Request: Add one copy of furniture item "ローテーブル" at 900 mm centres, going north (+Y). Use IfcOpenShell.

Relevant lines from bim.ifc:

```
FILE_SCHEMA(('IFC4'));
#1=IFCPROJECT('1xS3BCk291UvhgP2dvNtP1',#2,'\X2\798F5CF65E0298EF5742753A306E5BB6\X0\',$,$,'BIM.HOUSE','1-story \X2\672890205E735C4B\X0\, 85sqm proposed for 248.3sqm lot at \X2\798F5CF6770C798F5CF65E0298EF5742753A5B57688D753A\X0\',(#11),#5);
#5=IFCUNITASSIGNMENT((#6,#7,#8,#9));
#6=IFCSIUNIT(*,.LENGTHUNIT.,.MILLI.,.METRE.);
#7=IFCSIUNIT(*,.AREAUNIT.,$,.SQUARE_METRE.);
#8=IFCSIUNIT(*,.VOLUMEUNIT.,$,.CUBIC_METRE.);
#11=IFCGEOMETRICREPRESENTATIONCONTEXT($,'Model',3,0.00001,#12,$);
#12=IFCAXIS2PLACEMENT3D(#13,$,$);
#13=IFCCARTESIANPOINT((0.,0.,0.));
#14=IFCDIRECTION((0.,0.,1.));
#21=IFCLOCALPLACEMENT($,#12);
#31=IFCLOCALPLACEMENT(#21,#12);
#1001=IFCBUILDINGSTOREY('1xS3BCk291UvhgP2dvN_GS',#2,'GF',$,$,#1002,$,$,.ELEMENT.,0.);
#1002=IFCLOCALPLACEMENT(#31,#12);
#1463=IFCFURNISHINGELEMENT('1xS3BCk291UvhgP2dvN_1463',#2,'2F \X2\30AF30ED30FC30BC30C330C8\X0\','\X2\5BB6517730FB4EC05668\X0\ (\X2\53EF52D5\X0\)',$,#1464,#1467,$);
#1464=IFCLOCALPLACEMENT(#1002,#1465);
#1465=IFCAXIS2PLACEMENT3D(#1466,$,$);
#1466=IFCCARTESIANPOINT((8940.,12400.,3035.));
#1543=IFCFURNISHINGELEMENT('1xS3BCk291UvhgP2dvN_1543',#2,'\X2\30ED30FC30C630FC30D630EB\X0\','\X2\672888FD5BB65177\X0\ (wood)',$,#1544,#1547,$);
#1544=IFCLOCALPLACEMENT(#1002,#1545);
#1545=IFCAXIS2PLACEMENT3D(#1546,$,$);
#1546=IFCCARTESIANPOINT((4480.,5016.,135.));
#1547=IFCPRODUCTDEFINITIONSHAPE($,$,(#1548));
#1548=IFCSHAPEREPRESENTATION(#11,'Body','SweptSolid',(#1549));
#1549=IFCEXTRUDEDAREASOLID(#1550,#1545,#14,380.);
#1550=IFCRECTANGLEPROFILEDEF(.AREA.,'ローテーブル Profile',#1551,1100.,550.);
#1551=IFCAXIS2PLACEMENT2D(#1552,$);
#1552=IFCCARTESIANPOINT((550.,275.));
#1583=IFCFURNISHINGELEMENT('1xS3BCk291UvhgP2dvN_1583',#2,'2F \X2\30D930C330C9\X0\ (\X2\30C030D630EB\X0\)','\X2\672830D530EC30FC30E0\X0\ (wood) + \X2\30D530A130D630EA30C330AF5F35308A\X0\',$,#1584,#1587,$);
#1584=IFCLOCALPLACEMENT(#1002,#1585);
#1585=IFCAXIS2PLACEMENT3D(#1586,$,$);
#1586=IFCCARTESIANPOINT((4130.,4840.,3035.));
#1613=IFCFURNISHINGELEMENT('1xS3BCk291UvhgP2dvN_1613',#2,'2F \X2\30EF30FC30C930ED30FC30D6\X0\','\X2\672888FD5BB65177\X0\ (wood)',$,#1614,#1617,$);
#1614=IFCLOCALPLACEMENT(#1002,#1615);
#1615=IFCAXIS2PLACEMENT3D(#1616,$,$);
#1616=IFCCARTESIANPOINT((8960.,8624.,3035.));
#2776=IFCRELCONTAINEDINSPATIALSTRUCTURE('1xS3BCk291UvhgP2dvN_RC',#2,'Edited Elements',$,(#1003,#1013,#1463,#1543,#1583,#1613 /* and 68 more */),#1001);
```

```python
import numpy as np
import ifcopenshell
import ifcopenshell.api.geometry
import ifcopenshell.api.root
import ifcopenshell.util.element
import ifcopenshell.util.placement

model = ifcopenshell.open("bim.ifc")


def reuse_history(source, copy):
    """copy_class also copies each property set's owner history, people and application; keep the originals."""
    for rel in copy.IsDefinedBy:
        if rel.is_a("IfcRelDefinesByProperties") and (history := rel.RelatingPropertyDefinition.OwnerHistory):
            rel.RelatingPropertyDefinition.OwnerHistory = source.OwnerHistory
            ifcopenshell.util.element.remove_deep2(model, history)


source = model.by_guid("1xS3BCk291UvhgP2dvN_1543")
base = ifcopenshell.util.placement.get_local_placement(source.ObjectPlacement)
step = np.array([0.0, 1.0, 0.0]) * 900.0

for i in range(1, 2):
    copy = ifcopenshell.api.root.copy_class(model, product=source)
    copy.Representation = ifcopenshell.util.element.copy_deep(
        model, source.Representation, exclude=["IfcGeometricRepresentationContext", "IfcRepresentationMap"]
    )
    reuse_history(source, copy)
    matrix = base.copy()
    matrix[:3, 3] += i * step
    print("added at", matrix[:3, 3].round(3) + 0.0)
    ifcopenshell.api.geometry.edit_object_placement(model, product=copy, matrix=matrix, is_si=False)

model.write("bim_rev.ifc")
```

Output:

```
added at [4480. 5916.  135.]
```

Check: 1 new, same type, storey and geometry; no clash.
